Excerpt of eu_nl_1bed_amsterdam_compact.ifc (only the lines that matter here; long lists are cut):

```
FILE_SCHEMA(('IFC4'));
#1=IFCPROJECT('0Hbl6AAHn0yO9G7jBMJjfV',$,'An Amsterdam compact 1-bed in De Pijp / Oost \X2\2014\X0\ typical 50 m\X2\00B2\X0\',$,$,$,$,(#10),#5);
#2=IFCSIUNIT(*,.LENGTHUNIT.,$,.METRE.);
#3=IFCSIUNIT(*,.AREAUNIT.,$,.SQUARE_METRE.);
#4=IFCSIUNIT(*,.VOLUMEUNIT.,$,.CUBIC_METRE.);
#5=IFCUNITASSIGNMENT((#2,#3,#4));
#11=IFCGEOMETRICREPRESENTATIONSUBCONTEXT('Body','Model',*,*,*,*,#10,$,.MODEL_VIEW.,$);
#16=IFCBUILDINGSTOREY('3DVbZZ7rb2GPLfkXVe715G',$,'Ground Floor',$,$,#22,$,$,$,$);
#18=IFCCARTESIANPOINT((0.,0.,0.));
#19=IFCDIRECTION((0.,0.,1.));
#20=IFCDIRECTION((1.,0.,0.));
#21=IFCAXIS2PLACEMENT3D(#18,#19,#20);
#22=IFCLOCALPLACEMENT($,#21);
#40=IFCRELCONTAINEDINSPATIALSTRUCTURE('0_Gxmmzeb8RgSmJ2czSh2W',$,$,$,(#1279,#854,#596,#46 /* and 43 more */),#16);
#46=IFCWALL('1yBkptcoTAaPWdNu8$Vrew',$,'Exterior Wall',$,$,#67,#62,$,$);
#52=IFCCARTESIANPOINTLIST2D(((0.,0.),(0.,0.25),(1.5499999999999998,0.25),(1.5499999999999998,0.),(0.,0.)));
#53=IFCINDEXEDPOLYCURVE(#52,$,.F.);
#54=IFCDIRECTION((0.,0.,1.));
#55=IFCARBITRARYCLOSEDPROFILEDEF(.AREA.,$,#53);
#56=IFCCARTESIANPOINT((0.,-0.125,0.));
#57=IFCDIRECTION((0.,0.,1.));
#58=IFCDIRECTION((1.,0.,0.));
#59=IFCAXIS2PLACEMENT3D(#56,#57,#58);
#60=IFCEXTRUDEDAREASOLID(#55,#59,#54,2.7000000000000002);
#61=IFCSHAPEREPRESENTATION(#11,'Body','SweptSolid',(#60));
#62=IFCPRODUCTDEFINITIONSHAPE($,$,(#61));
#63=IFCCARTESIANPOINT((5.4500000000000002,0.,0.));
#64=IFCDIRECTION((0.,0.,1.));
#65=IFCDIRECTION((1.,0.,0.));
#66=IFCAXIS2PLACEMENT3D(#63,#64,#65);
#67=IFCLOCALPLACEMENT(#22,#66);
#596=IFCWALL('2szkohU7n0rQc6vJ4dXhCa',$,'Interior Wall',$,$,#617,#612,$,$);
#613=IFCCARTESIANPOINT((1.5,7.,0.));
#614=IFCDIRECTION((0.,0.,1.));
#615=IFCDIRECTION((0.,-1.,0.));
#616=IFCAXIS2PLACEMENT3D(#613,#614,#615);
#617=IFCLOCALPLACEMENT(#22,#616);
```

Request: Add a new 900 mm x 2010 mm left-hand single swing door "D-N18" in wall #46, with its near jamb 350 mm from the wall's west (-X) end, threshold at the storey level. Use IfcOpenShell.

```python
import numpy as np
import ifcopenshell
import ifcopenshell.api.feature
import ifcopenshell.api.geometry
import ifcopenshell.api.root
import ifcopenshell.api.spatial
import ifcopenshell.geom
import ifcopenshell.util.element
import ifcopenshell.util.placement
import ifcopenshell.util.representation
import ifcopenshell.util.shape
import ifcopenshell.util.unit

model = ifcopenshell.open("eu_nl_1bed_amsterdam_compact.ifc")
unit_scale = ifcopenshell.util.unit.calculate_unit_scale(model)
settings = ifcopenshell.geom.settings()


def volume(element):
    """Net volume in cubic metres, openings subtracted."""
    shape = ifcopenshell.geom.create_shape(settings, element)
    return ifcopenshell.util.shape.get_volume(shape.geometry)


wall = model.by_guid("1yBkptcoTAaPWdNu8$Vrew")
storey = ifcopenshell.util.element.get_container(wall, ifc_class="IfcBuildingStorey")
context = ifcopenshell.util.representation.get_context(model, "Model", "Body", "MODEL_VIEW")
before = volume(wall)

width, height, from_end, sill = 0.9, 2.01, 0.35, 0.0  # metres

# The wall runs along its own X axis, and the end named is its -X end.
wall_shape = ifcopenshell.geom.create_shape(settings, wall)
x, y, z = ifcopenshell.util.shape.get_vertices(wall_shape.geometry).T
start = x.min() + from_end
face, thickness = float(y.min()), float(y.max() - y.min())
wall_matrix = ifcopenshell.util.placement.get_local_placement(wall.ObjectPlacement)
level = ifcopenshell.util.placement.get_local_placement(storey.ObjectPlacement)[2, 3]


def in_wall(x, y):
    """Placement at x, y metres in the wall's axes, at sill height."""
    matrix = wall_matrix.copy()
    matrix[:, 3] = wall_matrix @ np.array([x / unit_scale, y / unit_scale, 0.0, 1.0])
    matrix[2, 3] = level + sill / unit_scale
    return matrix


# Opening: a box that overshoots both wall faces by 50 mm.
opening = ifcopenshell.api.root.create_entity(model, ifc_class="IfcOpeningElement", predefined_type="OPENING")
box = ifcopenshell.api.geometry.add_wall_representation(
    model, context=context, length=width, height=height, thickness=thickness + 0.1
)
ifcopenshell.api.geometry.assign_representation(model, product=opening, representation=box)
ifcopenshell.api.geometry.edit_object_placement(model, product=opening, matrix=in_wall(start, face - 0.05), is_si=False)
ifcopenshell.api.feature.add_feature(model, feature=opening, element=wall)

door = ifcopenshell.api.root.create_entity(model, ifc_class="IfcDoor", name="D-N18", predefined_type="DOOR")
door.OverallWidth, door.OverallHeight = width / unit_scale, height / unit_scale
door.OperationType = "SINGLE_SWING_LEFT"
body = ifcopenshell.api.geometry.add_door_representation(
    model,
    context=context,
    overall_width=door.OverallWidth,
    overall_height=door.OverallHeight,
    operation_type="SINGLE_SWING_LEFT",
    lining_properties={"LiningDepth": thickness / unit_scale, "ThresholdDepth": thickness / unit_scale},
)
ifcopenshell.api.geometry.assign_representation(model, product=door, representation=body)
ifcopenshell.api.spatial.assign_container(model, products=[door], relating_structure=storey)
ifcopenshell.api.feature.add_filling(model, opening=opening, element=door)

# The lining spans the wall, so the door starts at the wall face.
ifcopenshell.api.geometry.edit_object_placement(model, product=door, matrix=in_wall(start, face), is_si=False)

after = volume(wall)

print(f"wall volume {before:.3f} -> {after:.3f} m3")

model.write("eu_nl_1bed_amsterdam_compact_edited.ifc")
```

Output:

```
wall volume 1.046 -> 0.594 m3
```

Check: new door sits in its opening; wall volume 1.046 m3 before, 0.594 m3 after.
